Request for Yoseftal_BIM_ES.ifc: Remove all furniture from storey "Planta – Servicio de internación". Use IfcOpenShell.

First a look at what the model holds.

```python
import ifcopenshell
import ifcopenshell.util.element

model = ifcopenshell.open("Yoseftal_BIM_ES.ifc")
print(model.schema)
storey = next(s for s in model.by_type("IfcBuildingStorey") if s.Name == "Planta – Servicio de internación")
furniture = [e for e in ifcopenshell.util.element.get_decomposition(storey) if e.is_a("IfcFurnishingElement")]
seen = {}
for e in furniture:
    element_type = ifcopenshell.util.element.get_type(e)
    name = element_type.Name if element_type not in (None, e) else None
    seen[name] = seen.get(name, 0) + 1
for name, count in sorted(seen.items(), key=str):
    print(count, "x", name)
```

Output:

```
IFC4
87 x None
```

```python
import ifcopenshell
import ifcopenshell.api.root
import ifcopenshell.util.element

model = ifcopenshell.open("Yoseftal_BIM_ES.ifc")

storey = next(s for s in model.by_type("IfcBuildingStorey") if s.Name == "Planta – Servicio de internación")
furniture = [e for e in ifcopenshell.util.element.get_decomposition(storey) if e.is_a("IfcFurnishingElement")]

for e in furniture:
    ifcopenshell.api.root.remove_product(model, product=e)
print(len(furniture), "removed")

model.write("Yoseftal_BIM_ES-out.ifc")
```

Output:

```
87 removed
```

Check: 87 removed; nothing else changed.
